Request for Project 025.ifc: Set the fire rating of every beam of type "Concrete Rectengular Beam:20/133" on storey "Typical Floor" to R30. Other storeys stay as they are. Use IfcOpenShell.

First a look at what the model holds.

```python
import ifcopenshell
import ifcopenshell.util.element

model = ifcopenshell.open("Project 025.ifc")
print(model.schema)
storey = next(s for s in model.by_type("IfcBuildingStorey") if s.Name == "Typical Floor")
beams = [e for e in ifcopenshell.util.element.get_decomposition(storey) if e.is_a("IfcBeam")]
seen = {}
for e in beams:
    element_type = ifcopenshell.util.element.get_type(e)
    key = (element_type.Name if element_type != e and element_type else None, ifcopenshell.util.element.get_pset(e, "Pset_BeamCommon", "FireRating"))
    seen[key] = seen.get(key, 0) + 1
for (name, value), count in sorted(seen.items(), key=str):
    print(count, "x", name, "|", value)
```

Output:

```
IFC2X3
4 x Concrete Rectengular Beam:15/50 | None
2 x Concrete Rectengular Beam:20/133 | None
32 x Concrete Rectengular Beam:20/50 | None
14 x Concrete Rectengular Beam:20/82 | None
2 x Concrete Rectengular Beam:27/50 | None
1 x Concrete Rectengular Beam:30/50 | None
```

```python
import ifcopenshell
import ifcopenshell.api.pset
import ifcopenshell.util.element

model = ifcopenshell.open("Project 025.ifc")

storey = next(s for s in model.by_type("IfcBuildingStorey") if s.Name == "Typical Floor")
beams = [e for e in ifcopenshell.util.element.get_decomposition(storey) if e.is_a("IfcBeam")]

count = 0
for e in beams:
    element_type = ifcopenshell.util.element.get_type(e)
    if element_type in (None, e) or element_type.Name != "Concrete Rectengular Beam:20/133":
        continue
    # add_pset returns the element's existing set when there is one.
    pset = ifcopenshell.api.pset.add_pset(model, product=e, name="Pset_BeamCommon")
    ifcopenshell.api.pset.edit_pset(model, pset=pset, properties={"FireRating": "R30"})
    count += 1

print(count, "beams updated")

model.write("Project 025_updated.ifc")
```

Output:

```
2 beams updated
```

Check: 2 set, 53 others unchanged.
